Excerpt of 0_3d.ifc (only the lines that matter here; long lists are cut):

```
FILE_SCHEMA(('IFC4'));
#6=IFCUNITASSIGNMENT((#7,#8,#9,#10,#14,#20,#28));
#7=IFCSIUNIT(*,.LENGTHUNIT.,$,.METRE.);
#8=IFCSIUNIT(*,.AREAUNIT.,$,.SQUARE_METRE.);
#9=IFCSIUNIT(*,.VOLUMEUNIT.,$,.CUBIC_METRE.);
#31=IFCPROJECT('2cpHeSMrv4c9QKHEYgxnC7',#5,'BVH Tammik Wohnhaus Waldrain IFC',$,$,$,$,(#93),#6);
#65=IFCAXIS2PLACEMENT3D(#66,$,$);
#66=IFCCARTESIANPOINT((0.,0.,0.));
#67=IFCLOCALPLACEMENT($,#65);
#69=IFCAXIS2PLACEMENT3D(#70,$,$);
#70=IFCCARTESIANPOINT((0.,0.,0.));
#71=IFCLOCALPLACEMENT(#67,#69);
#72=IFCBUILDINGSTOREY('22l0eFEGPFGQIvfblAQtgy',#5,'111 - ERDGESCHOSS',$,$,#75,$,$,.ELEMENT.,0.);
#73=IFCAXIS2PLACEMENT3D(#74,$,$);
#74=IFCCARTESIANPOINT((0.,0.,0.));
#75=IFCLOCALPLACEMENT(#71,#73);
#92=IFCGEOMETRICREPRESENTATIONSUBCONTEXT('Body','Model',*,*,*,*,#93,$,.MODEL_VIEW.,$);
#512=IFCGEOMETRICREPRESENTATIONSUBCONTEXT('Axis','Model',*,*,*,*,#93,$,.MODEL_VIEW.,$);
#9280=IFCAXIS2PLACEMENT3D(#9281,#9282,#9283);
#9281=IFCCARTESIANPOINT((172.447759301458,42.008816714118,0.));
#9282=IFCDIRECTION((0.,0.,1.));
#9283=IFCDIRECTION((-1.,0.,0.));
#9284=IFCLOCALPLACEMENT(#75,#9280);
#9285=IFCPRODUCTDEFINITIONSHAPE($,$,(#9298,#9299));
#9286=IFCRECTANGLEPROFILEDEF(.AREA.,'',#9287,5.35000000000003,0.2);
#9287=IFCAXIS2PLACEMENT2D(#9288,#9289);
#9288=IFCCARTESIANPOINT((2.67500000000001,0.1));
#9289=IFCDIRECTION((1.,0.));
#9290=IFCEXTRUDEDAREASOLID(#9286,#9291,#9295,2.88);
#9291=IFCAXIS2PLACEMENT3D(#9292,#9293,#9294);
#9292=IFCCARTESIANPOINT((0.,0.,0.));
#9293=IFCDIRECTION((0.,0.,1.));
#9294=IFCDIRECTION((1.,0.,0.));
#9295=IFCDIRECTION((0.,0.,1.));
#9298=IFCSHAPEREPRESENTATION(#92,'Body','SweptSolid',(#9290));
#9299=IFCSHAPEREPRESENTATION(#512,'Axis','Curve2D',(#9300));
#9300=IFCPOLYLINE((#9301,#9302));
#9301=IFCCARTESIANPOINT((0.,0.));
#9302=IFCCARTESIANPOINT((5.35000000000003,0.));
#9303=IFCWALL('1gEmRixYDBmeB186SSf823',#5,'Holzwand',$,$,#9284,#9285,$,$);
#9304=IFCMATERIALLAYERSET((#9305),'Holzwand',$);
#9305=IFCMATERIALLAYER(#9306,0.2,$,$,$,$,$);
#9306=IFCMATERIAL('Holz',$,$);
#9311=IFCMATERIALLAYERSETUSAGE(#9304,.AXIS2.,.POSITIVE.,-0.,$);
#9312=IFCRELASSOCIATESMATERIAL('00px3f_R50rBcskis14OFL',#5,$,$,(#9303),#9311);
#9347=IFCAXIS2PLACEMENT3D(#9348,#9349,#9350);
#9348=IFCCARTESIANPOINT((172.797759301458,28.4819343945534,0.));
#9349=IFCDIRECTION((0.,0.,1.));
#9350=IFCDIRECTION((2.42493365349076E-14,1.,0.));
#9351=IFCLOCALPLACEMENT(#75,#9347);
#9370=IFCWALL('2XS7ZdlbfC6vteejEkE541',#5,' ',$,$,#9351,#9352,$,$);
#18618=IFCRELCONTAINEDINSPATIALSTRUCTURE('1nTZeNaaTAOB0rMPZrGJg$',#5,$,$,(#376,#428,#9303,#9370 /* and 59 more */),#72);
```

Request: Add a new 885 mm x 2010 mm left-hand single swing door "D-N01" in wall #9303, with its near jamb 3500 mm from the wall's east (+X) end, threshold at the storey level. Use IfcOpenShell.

```python
import numpy as np
import ifcopenshell
import ifcopenshell.api.feature
import ifcopenshell.api.geometry
import ifcopenshell.api.root
import ifcopenshell.api.spatial
import ifcopenshell.geom
import ifcopenshell.util.element
import ifcopenshell.util.placement
import ifcopenshell.util.representation
import ifcopenshell.util.shape
import ifcopenshell.util.unit

model = ifcopenshell.open("0_3d.ifc")
unit_scale = ifcopenshell.util.unit.calculate_unit_scale(model)
settings = ifcopenshell.geom.settings()


def volume(element):
    """Net volume in cubic metres, openings subtracted."""
    shape = ifcopenshell.geom.create_shape(settings, element)
    return ifcopenshell.util.shape.get_volume(shape.geometry)


wall = model.by_guid("1gEmRixYDBmeB186SSf823")
storey = ifcopenshell.util.element.get_container(wall, ifc_class="IfcBuildingStorey")
context = ifcopenshell.util.representation.get_context(model, "Model", "Body", "MODEL_VIEW")
before = volume(wall)

width, height, from_end, sill = 0.885, 2.01, 3.5, 0.0  # metres

# The wall runs along its own X axis, and the end named is its -X end.
wall_shape = ifcopenshell.geom.create_shape(settings, wall)
x, y, z = ifcopenshell.util.shape.get_vertices(wall_shape.geometry).T
start = x.min() + from_end
face, thickness = float(y.min()), float(y.max() - y.min())
wall_matrix = ifcopenshell.util.placement.get_local_placement(wall.ObjectPlacement)
level = ifcopenshell.util.placement.get_local_placement(storey.ObjectPlacement)[2, 3]


def in_wall(x, y):
    """Placement at x, y metres in the wall's axes, at sill height."""
    matrix = wall_matrix.copy()
    matrix[:, 3] = wall_matrix @ np.array([x / unit_scale, y / unit_scale, 0.0, 1.0])
    matrix[2, 3] = level + sill / unit_scale
    return matrix


# Opening: a box that overshoots both wall faces by 50 mm.
opening = ifcopenshell.api.root.create_entity(model, ifc_class="IfcOpeningElement", predefined_type="OPENING")
box = ifcopenshell.api.geometry.add_wall_representation(
    model, context=context, length=width, height=height, thickness=thickness + 0.1
)
ifcopenshell.api.geometry.assign_representation(model, product=opening, representation=box)
ifcopenshell.api.geometry.edit_object_placement(model, product=opening, matrix=in_wall(start, face - 0.05), is_si=False)
ifcopenshell.api.feature.add_feature(model, feature=opening, element=wall)

door = ifcopenshell.api.root.create_entity(model, ifc_class="IfcDoor", name="D-N01", predefined_type="DOOR")
door.OverallWidth, door.OverallHeight = width / unit_scale, height / unit_scale
door.OperationType = "SINGLE_SWING_LEFT"
body = ifcopenshell.api.geometry.add_door_representation(
    model,
    context=context,
    overall_width=door.OverallWidth,
    overall_height=door.OverallHeight,
    operation_type="SINGLE_SWING_LEFT",
    lining_properties={"LiningDepth": thickness / unit_scale, "ThresholdDepth": thickness / unit_scale},
)
ifcopenshell.api.geometry.assign_representation(model, product=door, representation=body)
ifcopenshell.api.spatial.assign_container(model, products=[door], relating_structure=storey)
ifcopenshell.api.feature.add_filling(model, opening=opening, element=door)

# The lining spans the wall, so the door starts at the wall face.
ifcopenshell.api.geometry.edit_object_placement(model, product=door, matrix=in_wall(start, face), is_si=False)

after = volume(wall)

print(f"wall volume {before:.3f} -> {after:.3f} m3")

model.write("0_3d_v2.ifc")
```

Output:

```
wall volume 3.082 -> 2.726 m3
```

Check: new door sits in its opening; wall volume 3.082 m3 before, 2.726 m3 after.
